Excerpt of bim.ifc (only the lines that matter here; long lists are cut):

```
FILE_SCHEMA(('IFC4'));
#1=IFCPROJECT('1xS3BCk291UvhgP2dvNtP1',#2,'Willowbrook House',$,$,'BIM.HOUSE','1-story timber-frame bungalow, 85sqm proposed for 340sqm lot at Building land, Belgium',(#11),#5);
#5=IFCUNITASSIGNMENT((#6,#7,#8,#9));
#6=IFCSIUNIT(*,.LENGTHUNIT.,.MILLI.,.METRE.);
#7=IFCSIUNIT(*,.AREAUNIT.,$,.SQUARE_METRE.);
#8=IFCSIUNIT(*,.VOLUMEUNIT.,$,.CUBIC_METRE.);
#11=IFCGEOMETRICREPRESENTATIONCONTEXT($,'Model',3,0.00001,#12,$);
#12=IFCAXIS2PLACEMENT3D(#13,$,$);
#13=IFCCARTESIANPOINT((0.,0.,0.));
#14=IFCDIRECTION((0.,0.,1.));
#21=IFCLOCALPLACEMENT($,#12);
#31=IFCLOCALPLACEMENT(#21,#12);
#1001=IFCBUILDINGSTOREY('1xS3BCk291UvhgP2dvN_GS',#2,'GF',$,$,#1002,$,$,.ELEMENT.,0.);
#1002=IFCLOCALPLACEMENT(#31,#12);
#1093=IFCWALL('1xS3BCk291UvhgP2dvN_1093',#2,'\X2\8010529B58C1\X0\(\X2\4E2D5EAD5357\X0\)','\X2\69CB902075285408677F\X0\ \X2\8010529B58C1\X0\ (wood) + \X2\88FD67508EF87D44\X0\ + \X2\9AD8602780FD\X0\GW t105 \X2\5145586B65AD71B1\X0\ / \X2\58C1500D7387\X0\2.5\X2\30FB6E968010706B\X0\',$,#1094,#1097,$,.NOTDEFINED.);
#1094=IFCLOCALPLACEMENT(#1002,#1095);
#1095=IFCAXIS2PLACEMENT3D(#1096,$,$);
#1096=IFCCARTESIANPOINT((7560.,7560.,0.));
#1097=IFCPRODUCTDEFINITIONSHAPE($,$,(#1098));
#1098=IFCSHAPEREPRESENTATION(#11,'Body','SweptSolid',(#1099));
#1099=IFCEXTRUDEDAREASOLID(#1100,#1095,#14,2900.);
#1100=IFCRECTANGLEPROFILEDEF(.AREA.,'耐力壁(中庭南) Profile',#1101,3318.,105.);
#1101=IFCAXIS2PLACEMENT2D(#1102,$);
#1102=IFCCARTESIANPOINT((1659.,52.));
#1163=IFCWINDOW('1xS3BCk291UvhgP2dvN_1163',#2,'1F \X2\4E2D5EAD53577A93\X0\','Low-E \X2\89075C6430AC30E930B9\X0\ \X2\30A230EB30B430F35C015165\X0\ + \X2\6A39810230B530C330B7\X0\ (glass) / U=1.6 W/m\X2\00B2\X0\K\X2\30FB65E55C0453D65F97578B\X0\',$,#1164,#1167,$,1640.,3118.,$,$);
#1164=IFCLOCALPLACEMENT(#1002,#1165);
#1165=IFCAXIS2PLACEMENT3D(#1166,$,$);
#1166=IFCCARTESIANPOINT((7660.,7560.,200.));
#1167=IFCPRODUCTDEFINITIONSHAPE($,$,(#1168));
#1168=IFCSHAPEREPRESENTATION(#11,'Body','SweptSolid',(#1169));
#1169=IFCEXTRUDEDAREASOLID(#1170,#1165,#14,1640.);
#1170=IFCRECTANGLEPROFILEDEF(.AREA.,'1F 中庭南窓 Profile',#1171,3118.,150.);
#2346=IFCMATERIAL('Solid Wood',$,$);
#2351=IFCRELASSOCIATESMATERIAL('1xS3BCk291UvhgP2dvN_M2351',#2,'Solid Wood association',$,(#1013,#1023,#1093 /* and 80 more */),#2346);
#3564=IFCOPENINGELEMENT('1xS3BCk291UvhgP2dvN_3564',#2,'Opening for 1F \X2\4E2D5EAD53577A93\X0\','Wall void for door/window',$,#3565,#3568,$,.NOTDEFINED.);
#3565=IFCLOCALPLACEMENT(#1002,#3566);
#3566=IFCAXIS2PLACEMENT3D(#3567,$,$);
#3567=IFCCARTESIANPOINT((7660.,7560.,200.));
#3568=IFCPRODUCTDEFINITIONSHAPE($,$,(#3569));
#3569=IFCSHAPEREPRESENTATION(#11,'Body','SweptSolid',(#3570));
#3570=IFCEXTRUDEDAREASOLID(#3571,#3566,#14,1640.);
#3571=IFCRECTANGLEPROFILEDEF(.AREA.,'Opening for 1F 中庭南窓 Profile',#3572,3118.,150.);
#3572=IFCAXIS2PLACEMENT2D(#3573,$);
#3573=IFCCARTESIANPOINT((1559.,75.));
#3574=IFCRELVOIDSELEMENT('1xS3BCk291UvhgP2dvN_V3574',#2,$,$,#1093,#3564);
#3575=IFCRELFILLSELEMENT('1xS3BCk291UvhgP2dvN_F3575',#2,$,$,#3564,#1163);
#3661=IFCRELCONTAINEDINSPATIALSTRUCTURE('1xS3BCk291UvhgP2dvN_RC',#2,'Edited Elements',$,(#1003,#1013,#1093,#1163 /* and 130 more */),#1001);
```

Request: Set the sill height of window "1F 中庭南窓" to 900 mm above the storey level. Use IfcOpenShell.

```python
import numpy as np
import ifcopenshell
import ifcopenshell.api.geometry
import ifcopenshell.geom
import ifcopenshell.util.element
import ifcopenshell.util.placement
import ifcopenshell.util.shape
import ifcopenshell.util.unit

model = ifcopenshell.open("bim.ifc")
unit_scale = ifcopenshell.util.unit.calculate_unit_scale(model)

window = model.by_guid("1xS3BCk291UvhgP2dvN_1163")
opening = window.FillsVoids[0].RelatingOpeningElement
storey = ifcopenshell.util.element.get_container(window, ifc_class="IfcBuildingStorey")
level = ifcopenshell.util.placement.get_local_placement(storey.ObjectPlacement)[2, 3]

# The opening's origin need not be at the sill, so measure its lowest point.
shape = ifcopenshell.geom.create_shape(ifcopenshell.geom.settings(), opening)
bottom = ifcopenshell.util.shape.get_shape_bottom_elevation(shape, shape.geometry) / unit_scale
dz = level + 0.9 / unit_scale - bottom

shift = np.array([0.0, 0.0, dz])
# The window is not placed relative to its opening, so move both.
for product in (opening, window):
    matrix = ifcopenshell.util.placement.get_local_placement(product.ObjectPlacement)
    matrix[:3, 3] += shift
    ifcopenshell.api.geometry.edit_object_placement(model, product=product, matrix=matrix, is_si=False)

print(f"moved by {dz * unit_scale:+.3f} m")

model.write("bim_edited.ifc")
```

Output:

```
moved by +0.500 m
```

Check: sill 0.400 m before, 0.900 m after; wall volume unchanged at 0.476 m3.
